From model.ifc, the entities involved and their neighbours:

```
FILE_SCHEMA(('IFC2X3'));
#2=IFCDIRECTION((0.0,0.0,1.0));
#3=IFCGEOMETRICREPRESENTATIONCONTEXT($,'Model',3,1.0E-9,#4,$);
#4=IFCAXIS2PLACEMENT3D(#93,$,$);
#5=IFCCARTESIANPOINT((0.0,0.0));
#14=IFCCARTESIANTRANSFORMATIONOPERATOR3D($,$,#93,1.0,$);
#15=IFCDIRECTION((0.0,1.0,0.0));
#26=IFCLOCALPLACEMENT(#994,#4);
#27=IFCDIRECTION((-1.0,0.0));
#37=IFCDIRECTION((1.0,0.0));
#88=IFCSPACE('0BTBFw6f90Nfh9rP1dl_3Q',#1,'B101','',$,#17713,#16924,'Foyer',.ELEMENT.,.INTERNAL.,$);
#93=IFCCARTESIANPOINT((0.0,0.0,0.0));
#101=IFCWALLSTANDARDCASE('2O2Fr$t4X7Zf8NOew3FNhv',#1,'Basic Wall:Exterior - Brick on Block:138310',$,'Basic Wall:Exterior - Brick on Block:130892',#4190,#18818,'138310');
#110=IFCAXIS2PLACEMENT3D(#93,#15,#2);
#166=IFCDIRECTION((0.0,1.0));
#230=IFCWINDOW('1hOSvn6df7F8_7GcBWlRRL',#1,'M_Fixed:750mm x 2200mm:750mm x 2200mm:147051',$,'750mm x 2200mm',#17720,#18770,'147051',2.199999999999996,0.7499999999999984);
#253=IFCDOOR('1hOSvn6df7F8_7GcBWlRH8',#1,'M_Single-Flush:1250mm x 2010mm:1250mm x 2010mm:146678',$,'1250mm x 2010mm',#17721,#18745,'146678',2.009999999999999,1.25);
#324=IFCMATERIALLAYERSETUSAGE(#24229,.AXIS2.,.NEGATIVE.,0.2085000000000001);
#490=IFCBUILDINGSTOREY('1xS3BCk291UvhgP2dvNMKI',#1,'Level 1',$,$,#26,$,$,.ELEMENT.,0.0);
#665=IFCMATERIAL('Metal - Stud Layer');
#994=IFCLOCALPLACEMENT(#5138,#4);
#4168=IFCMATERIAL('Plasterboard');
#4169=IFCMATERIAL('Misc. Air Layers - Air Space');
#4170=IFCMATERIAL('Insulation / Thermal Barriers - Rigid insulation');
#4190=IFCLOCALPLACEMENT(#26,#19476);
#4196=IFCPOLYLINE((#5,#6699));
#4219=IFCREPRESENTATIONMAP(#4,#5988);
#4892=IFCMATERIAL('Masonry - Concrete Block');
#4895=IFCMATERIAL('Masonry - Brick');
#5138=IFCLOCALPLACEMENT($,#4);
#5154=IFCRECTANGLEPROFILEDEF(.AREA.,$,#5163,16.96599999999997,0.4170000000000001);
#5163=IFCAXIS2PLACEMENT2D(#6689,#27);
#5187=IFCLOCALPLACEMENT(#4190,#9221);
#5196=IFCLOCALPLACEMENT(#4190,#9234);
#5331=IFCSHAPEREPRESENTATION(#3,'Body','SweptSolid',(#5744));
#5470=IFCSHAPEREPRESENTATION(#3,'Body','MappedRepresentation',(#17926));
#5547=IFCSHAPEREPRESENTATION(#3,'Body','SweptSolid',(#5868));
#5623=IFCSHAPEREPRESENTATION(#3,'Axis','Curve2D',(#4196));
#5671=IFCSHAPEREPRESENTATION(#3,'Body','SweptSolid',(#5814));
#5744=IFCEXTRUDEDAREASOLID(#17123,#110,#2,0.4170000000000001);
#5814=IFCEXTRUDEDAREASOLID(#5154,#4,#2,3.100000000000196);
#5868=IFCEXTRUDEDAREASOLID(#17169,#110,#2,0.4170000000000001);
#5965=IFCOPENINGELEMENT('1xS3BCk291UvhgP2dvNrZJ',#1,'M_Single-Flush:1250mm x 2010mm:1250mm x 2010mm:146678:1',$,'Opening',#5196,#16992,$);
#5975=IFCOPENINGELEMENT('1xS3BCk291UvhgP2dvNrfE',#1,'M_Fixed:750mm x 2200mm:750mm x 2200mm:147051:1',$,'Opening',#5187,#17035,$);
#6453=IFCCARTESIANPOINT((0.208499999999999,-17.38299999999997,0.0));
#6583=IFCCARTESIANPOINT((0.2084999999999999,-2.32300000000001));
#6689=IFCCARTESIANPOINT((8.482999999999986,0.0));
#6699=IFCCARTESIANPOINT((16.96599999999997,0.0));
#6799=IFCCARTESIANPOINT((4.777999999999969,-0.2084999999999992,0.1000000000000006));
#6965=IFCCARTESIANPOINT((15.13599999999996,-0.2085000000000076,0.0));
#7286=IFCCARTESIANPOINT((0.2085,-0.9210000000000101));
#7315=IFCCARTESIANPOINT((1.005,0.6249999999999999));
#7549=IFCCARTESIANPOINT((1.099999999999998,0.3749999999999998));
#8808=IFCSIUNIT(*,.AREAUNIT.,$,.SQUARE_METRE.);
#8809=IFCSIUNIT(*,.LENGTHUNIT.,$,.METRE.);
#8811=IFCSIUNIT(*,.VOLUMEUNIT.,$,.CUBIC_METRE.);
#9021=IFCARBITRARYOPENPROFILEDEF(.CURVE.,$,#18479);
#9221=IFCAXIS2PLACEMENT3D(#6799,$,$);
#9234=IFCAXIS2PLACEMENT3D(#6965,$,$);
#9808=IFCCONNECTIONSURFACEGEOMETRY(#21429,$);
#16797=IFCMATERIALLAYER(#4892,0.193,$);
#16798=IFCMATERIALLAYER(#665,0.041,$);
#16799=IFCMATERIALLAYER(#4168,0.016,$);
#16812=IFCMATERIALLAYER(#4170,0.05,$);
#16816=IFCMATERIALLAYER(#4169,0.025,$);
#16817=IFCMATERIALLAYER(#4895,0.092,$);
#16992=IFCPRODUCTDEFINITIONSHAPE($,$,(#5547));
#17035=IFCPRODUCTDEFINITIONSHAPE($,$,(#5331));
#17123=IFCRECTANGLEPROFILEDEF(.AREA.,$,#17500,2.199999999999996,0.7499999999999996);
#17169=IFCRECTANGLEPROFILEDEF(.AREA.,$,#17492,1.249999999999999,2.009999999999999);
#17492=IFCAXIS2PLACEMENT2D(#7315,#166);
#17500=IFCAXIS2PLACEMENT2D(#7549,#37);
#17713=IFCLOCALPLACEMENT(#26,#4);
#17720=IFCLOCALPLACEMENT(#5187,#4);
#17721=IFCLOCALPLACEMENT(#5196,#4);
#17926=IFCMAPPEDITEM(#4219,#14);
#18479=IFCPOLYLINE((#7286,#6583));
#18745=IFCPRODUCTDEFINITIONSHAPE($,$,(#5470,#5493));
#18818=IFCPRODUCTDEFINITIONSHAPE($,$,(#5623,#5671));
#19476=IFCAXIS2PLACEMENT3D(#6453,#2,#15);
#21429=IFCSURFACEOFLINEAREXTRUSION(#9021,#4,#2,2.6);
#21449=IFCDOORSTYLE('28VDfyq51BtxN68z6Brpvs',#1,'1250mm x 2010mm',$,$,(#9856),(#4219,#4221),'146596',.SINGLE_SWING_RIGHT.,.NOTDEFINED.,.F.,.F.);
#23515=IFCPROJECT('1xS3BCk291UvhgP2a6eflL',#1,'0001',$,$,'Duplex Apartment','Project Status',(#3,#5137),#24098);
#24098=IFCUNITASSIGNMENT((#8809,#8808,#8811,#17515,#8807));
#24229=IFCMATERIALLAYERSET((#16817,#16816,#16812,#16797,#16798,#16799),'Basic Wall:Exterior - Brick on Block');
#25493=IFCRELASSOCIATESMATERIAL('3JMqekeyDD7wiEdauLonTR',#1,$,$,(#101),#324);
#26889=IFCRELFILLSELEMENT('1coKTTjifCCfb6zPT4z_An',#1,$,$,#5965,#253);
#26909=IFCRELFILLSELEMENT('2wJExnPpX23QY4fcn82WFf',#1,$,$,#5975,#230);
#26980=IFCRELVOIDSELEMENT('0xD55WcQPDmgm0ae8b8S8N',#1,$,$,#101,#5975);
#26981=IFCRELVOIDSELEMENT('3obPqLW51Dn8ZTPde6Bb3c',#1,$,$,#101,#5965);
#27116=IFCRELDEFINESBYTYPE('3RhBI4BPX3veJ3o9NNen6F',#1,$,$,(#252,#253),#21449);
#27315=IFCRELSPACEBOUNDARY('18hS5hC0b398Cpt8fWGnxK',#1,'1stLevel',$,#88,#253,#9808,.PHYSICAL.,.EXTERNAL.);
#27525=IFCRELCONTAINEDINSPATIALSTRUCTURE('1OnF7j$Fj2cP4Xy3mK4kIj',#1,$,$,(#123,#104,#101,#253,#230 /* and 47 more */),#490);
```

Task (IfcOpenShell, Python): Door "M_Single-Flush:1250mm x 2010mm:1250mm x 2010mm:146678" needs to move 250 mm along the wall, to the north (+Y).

```python
import numpy as np
import ifcopenshell
import ifcopenshell.api.geometry
import ifcopenshell.util.placement
import ifcopenshell.util.unit

model = ifcopenshell.open("model.ifc")
unit_scale = ifcopenshell.util.unit.calculate_unit_scale(model)

door = model.by_id(253)
opening = door.FillsVoids[0].RelatingOpeningElement
wall = opening.VoidsElements[0].RelatingBuildingElement

wall_matrix = ifcopenshell.util.placement.get_local_placement(wall.ObjectPlacement)
shift = wall_matrix[:3, 0] * 0.25 / unit_scale
before = ifcopenshell.util.placement.get_local_placement(door.ObjectPlacement)[:3, 3].copy()

# The door is placed relative to its opening, so it follows when the opening moves.
matrix = ifcopenshell.util.placement.get_local_placement(opening.ObjectPlacement)
matrix[:3, 3] += shift
ifcopenshell.api.geometry.edit_object_placement(
    model, product=opening, matrix=matrix, is_si=False, should_transform_children=True
)

# Space boundary surfaces are stored in each space's coordinates; move them too.
for rel in door.ProvidesBoundaries:
    if not rel.ConnectionGeometry:
        continue
    surface = rel.ConnectionGeometry.SurfaceOnRelatingElement
    space_matrix = ifcopenshell.util.placement.get_local_placement(rel.RelatingSpace.ObjectPlacement)
    point = np.array(surface.Position.Location.Coordinates) + space_matrix[:3, :3].T @ shift
    surface.Position = model.createIfcAxis2Placement3D(
        model.createIfcCartesianPoint(point.tolist()), surface.Position.Axis, surface.Position.RefDirection
    )

after = ifcopenshell.util.placement.get_local_placement(door.ObjectPlacement)[:3, 3]
print("door moved by", (after - before).round(3) + 0.0)

model.write("model_updated.ifc")
```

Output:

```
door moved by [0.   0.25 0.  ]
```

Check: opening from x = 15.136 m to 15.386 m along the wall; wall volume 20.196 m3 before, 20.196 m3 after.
